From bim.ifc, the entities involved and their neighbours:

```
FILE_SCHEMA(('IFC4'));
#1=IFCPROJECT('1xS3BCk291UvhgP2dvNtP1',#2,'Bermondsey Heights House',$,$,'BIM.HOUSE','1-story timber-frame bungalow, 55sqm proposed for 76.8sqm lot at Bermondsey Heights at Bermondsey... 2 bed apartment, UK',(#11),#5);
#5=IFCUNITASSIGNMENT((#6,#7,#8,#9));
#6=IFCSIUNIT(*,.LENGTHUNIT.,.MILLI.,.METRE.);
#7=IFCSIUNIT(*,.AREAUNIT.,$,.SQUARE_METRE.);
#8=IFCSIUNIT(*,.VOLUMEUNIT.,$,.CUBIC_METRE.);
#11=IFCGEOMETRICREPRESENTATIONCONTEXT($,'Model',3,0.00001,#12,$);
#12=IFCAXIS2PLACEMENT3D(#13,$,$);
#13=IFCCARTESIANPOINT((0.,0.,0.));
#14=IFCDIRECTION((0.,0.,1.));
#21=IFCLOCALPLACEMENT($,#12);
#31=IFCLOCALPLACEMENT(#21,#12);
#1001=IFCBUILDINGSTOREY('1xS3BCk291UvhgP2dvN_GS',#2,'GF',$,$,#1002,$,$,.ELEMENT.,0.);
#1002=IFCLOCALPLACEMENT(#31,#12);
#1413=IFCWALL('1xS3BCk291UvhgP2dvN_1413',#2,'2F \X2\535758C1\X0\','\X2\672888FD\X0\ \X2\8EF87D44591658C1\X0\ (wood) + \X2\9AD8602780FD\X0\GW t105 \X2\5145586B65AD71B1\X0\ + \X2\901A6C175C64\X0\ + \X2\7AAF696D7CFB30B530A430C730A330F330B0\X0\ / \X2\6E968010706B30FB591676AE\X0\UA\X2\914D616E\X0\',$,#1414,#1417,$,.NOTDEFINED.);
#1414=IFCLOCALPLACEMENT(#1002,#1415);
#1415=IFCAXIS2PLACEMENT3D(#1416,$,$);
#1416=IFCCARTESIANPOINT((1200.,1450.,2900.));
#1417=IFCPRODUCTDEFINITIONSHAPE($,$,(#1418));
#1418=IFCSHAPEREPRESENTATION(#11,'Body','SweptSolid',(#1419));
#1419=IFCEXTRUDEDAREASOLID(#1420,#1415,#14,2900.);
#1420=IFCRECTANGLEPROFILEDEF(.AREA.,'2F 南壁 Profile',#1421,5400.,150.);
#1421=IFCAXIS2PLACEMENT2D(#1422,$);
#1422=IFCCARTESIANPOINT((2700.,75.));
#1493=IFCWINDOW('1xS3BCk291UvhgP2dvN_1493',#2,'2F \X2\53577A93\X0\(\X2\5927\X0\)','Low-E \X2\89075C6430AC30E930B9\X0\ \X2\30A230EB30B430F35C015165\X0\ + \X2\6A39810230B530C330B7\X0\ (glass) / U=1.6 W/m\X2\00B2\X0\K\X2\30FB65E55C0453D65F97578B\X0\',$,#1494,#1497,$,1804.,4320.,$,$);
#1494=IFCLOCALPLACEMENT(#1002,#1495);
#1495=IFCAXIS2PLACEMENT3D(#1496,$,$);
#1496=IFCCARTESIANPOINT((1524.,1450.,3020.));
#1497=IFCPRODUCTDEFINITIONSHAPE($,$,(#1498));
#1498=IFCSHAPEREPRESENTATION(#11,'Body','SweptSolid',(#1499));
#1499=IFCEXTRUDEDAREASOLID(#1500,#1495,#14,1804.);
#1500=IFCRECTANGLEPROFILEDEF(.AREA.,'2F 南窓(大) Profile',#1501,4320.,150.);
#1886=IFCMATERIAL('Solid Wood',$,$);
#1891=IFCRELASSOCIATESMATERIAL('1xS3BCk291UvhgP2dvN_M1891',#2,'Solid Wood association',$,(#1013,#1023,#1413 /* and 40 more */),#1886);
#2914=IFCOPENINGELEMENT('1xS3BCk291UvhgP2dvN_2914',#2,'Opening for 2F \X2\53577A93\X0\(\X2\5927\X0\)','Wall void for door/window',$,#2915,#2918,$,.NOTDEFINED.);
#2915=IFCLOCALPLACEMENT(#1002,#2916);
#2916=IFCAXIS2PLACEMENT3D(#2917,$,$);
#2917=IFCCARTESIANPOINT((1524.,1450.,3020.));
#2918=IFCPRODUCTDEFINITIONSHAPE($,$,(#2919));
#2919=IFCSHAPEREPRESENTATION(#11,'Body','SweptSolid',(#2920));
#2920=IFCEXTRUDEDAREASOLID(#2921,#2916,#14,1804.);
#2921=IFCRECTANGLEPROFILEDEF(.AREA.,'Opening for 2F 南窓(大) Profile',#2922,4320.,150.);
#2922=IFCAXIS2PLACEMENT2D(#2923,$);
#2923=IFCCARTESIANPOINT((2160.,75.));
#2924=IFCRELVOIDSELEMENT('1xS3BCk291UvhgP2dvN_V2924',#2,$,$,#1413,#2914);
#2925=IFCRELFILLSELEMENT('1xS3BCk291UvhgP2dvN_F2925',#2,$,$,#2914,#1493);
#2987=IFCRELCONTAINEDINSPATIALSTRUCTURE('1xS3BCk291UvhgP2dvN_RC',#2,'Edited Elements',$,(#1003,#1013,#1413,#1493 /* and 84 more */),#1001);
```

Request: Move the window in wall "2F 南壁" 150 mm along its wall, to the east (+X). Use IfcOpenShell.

```python
import ifcopenshell
import ifcopenshell.api.geometry
import ifcopenshell.util.placement
import ifcopenshell.util.unit

model = ifcopenshell.open("bim.ifc")
unit_scale = ifcopenshell.util.unit.calculate_unit_scale(model)

window = model.by_guid("1xS3BCk291UvhgP2dvN_1493")
opening = window.FillsVoids[0].RelatingOpeningElement
wall = opening.VoidsElements[0].RelatingBuildingElement

wall_matrix = ifcopenshell.util.placement.get_local_placement(wall.ObjectPlacement)
shift = wall_matrix[:3, 0] * 0.15 / unit_scale
before = ifcopenshell.util.placement.get_local_placement(window.ObjectPlacement)[:3, 3].copy()

# The window is not placed relative to its opening, so move both.
for product in (opening, window):
    matrix = ifcopenshell.util.placement.get_local_placement(product.ObjectPlacement)
    matrix[:3, 3] += shift
    ifcopenshell.api.geometry.edit_object_placement(model, product=product, matrix=matrix, is_si=False)

after = ifcopenshell.util.placement.get_local_placement(window.ObjectPlacement)[:3, 3]
print("window moved by", (after - before).round(3) + 0.0)

model.write("bim_v2.ifc")
```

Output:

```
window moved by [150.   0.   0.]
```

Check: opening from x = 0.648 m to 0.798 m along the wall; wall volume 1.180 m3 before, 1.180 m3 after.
